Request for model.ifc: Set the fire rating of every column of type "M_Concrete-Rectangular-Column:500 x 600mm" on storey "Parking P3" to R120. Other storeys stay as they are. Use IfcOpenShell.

First a look at what the model holds.

```python
import ifcopenshell
import ifcopenshell.util.element

model = ifcopenshell.open("model.ifc")
print(model.schema)
storey = next(s for s in model.by_type("IfcBuildingStorey") if s.Name == "Parking P3")
columns = [e for e in ifcopenshell.util.element.get_decomposition(storey) if e.is_a("IfcColumn")]
seen = {}
for e in columns:
    element_type = ifcopenshell.util.element.get_type(e)
    key = (element_type.Name if element_type != e and element_type else None, ifcopenshell.util.element.get_pset(e, "Pset_ColumnCommon", "FireRating"))
    seen[key] = seen.get(key, 0) + 1
for (name, value), count in sorted(seen.items(), key=str):
    print(count, "x", name, "|", value)
```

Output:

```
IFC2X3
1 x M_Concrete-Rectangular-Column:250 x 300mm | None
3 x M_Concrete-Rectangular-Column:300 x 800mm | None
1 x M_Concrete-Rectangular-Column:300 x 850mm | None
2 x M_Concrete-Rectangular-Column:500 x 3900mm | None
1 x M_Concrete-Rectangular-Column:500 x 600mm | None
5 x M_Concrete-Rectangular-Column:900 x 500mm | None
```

```python
import ifcopenshell
import ifcopenshell.api.pset
import ifcopenshell.util.element

model = ifcopenshell.open("model.ifc")

storey = next(s for s in model.by_type("IfcBuildingStorey") if s.Name == "Parking P3")
columns = [e for e in ifcopenshell.util.element.get_decomposition(storey) if e.is_a("IfcColumn")]

count = 0
for e in columns:
    element_type = ifcopenshell.util.element.get_type(e)
    if element_type in (None, e) or element_type.Name != "M_Concrete-Rectangular-Column:500 x 600mm":
        continue
    # add_pset returns the element's existing set when there is one.
    pset = ifcopenshell.api.pset.add_pset(model, product=e, name="Pset_ColumnCommon")
    ifcopenshell.api.pset.edit_pset(model, pset=pset, properties={"FireRating": "R120"})
    count += 1

print(count, "columns updated")

model.write("model-out.ifc")
```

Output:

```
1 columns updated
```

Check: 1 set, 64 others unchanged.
